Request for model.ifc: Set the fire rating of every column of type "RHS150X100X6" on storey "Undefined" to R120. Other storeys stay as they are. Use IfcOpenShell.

First a look at what the model holds.

```python
import ifcopenshell
import ifcopenshell.util.element

model = ifcopenshell.open("model.ifc")
print(model.schema)
storey = next(s for s in model.by_type("IfcBuildingStorey") if s.Name == "Undefined")
columns = [e for e in ifcopenshell.util.element.get_decomposition(storey) if e.is_a("IfcColumn")]
seen = {}
for e in columns:
    element_type = ifcopenshell.util.element.get_type(e)
    key = (element_type.Name if element_type != e and element_type else None, ifcopenshell.util.element.get_pset(e, "Pset_ColumnCommon", "FireRating"))
    seen[key] = seen.get(key, 0) + 1
for (name, value), count in sorted(seen.items(), key=str):
    print(count, "x", name, "|", value)
```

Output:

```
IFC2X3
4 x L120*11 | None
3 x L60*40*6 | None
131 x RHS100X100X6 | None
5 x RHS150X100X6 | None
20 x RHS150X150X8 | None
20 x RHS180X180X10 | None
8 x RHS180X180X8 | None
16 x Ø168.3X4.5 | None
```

```python
import ifcopenshell
import ifcopenshell.api.pset
import ifcopenshell.util.element

model = ifcopenshell.open("model.ifc")

storey = next(s for s in model.by_type("IfcBuildingStorey") if s.Name == "Undefined")
columns = [e for e in ifcopenshell.util.element.get_decomposition(storey) if e.is_a("IfcColumn")]

count = 0
for e in columns:
    element_type = ifcopenshell.util.element.get_type(e)
    if element_type in (None, e) or element_type.Name != "RHS150X100X6":
        continue
    found = ifcopenshell.util.element.get_pset(e, "Pset_ColumnCommon", should_inherit=False)
    if found:
        pset = model.by_id(found["id"])
        if len(ifcopenshell.util.element.get_elements_by_pset(pset)) > 1:
            pset = ifcopenshell.api.pset.unshare_pset(model, products=[e], pset=pset)[0]
    else:
        pset = ifcopenshell.api.pset.add_pset(model, product=e, name="Pset_ColumnCommon")
    ifcopenshell.api.pset.edit_pset(model, pset=pset, properties={"FireRating": "R120"})
    count += 1

print(count, "columns updated")

model.write("model_edited.ifc")
```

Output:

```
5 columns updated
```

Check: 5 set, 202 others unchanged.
